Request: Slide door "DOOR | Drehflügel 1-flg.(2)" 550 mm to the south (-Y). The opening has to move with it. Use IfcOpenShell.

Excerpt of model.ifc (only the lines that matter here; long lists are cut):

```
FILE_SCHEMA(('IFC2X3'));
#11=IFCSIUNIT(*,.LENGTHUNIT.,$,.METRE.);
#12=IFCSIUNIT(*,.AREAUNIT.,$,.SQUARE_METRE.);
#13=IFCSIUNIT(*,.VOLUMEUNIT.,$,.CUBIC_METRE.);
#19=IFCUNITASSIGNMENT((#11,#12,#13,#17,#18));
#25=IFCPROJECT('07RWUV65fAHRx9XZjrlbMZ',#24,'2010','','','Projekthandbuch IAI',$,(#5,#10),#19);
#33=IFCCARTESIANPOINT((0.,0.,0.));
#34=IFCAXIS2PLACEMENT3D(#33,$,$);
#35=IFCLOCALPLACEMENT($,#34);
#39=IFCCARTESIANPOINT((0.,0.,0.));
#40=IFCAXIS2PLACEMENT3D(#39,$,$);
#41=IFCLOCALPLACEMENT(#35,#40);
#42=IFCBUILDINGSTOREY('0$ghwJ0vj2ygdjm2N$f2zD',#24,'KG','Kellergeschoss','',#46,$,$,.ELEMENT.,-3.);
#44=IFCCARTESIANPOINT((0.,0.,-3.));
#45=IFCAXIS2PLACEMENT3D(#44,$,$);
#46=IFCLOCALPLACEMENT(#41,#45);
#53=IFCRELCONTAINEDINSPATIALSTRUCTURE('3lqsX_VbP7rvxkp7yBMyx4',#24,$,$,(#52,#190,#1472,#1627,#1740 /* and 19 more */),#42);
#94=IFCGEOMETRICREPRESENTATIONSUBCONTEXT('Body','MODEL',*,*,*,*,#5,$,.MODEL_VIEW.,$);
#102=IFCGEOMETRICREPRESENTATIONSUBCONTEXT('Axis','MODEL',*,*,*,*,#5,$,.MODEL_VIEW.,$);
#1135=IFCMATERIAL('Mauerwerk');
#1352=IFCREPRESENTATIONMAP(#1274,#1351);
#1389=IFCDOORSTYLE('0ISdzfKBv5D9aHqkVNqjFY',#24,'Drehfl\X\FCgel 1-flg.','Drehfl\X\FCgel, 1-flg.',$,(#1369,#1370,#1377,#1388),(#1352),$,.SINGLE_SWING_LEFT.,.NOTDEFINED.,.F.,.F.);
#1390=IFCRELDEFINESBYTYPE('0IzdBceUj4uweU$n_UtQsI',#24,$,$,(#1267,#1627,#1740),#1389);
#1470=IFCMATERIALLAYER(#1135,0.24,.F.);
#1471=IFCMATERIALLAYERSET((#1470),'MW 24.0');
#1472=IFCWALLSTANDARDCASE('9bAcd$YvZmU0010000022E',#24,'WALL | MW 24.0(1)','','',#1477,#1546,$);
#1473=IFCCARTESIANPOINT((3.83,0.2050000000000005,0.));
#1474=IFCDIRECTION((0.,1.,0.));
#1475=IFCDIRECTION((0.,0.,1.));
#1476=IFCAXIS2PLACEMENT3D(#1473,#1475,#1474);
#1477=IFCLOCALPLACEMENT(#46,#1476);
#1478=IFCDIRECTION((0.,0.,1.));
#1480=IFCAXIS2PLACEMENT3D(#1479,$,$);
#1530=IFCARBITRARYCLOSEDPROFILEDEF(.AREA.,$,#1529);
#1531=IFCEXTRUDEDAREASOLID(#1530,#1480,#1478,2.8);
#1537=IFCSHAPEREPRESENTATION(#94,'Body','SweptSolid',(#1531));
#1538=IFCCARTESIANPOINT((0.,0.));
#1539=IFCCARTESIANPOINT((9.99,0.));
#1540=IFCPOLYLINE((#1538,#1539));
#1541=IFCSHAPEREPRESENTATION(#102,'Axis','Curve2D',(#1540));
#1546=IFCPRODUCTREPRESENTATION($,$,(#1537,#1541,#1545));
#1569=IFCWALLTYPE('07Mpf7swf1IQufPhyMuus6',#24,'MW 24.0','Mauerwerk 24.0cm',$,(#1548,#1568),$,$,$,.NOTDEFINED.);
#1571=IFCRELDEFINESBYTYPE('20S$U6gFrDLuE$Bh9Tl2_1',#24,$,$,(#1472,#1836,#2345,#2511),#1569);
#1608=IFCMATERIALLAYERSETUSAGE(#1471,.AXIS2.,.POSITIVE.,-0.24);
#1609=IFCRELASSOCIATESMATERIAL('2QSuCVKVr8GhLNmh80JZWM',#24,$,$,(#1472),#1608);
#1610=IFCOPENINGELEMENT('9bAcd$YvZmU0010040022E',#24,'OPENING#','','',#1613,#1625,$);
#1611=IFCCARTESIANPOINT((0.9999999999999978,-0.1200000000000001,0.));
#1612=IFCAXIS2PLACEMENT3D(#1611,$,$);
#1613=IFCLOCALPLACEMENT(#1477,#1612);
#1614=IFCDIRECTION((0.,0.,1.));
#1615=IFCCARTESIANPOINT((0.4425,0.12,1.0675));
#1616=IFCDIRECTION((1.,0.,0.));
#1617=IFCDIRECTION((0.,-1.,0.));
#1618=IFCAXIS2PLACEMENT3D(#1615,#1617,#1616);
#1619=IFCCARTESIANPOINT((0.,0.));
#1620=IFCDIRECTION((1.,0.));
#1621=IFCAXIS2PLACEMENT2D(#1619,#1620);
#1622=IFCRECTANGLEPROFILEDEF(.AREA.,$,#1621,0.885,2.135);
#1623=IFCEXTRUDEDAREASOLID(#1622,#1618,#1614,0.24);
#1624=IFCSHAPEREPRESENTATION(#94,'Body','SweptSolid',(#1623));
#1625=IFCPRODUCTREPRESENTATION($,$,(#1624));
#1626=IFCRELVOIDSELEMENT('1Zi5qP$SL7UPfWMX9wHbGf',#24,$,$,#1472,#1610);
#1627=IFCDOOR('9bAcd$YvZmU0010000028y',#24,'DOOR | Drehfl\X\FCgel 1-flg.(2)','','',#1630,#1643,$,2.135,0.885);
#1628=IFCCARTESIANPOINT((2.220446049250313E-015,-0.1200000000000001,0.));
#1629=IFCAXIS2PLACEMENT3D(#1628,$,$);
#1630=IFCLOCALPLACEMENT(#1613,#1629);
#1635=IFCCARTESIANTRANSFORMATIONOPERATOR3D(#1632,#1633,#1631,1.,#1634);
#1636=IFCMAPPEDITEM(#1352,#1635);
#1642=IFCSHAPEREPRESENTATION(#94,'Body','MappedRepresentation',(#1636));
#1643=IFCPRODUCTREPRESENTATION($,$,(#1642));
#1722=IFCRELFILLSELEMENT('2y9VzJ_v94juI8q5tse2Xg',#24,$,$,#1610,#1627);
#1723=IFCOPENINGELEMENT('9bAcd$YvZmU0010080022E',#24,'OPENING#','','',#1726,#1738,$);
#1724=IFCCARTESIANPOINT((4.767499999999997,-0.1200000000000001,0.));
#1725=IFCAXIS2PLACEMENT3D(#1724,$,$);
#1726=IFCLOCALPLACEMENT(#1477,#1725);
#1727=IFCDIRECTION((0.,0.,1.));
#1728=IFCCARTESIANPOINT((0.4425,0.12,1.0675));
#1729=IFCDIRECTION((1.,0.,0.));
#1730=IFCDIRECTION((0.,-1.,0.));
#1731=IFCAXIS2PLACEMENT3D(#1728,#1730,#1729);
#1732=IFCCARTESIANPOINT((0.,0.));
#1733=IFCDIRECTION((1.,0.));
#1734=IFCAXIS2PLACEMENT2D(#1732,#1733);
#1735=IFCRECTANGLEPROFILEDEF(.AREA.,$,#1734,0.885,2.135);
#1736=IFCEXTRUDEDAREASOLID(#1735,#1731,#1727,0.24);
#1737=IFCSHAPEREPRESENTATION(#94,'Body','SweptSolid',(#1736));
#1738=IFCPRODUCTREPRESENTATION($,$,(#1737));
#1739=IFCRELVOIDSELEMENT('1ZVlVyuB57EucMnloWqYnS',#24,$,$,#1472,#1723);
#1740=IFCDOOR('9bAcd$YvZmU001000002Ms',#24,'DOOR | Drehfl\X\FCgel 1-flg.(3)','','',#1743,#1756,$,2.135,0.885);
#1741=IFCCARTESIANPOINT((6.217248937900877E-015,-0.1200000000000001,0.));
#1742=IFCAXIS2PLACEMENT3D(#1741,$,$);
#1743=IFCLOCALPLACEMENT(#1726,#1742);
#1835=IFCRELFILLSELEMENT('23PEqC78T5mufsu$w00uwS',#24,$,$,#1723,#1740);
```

```python
import ifcopenshell
import ifcopenshell.api.geometry
import ifcopenshell.util.placement

model = ifcopenshell.open("model.ifc")

door = model.by_guid("9bAcd$YvZmU0010000028y")
opening = door.FillsVoids[0].RelatingOpeningElement
wall = opening.VoidsElements[0].RelatingBuildingElement

wall_matrix = ifcopenshell.util.placement.get_local_placement(wall.ObjectPlacement)
shift = wall_matrix[:3, 0] * -0.55
before = ifcopenshell.util.placement.get_local_placement(door.ObjectPlacement)[:3, 3].copy()

# The door is placed relative to its opening, so it follows when the opening moves.
matrix = ifcopenshell.util.placement.get_local_placement(opening.ObjectPlacement)
matrix[:3, 3] += shift
ifcopenshell.api.geometry.edit_object_placement(
    model, product=opening, matrix=matrix, is_si=False, should_transform_children=True
)

after = ifcopenshell.util.placement.get_local_placement(door.ObjectPlacement)[:3, 3]
print("door moved by", (after - before).round(3) + 0.0)

model.write("model_v2.ifc")
```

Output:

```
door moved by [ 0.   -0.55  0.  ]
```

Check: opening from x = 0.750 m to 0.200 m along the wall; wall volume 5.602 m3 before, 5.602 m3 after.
